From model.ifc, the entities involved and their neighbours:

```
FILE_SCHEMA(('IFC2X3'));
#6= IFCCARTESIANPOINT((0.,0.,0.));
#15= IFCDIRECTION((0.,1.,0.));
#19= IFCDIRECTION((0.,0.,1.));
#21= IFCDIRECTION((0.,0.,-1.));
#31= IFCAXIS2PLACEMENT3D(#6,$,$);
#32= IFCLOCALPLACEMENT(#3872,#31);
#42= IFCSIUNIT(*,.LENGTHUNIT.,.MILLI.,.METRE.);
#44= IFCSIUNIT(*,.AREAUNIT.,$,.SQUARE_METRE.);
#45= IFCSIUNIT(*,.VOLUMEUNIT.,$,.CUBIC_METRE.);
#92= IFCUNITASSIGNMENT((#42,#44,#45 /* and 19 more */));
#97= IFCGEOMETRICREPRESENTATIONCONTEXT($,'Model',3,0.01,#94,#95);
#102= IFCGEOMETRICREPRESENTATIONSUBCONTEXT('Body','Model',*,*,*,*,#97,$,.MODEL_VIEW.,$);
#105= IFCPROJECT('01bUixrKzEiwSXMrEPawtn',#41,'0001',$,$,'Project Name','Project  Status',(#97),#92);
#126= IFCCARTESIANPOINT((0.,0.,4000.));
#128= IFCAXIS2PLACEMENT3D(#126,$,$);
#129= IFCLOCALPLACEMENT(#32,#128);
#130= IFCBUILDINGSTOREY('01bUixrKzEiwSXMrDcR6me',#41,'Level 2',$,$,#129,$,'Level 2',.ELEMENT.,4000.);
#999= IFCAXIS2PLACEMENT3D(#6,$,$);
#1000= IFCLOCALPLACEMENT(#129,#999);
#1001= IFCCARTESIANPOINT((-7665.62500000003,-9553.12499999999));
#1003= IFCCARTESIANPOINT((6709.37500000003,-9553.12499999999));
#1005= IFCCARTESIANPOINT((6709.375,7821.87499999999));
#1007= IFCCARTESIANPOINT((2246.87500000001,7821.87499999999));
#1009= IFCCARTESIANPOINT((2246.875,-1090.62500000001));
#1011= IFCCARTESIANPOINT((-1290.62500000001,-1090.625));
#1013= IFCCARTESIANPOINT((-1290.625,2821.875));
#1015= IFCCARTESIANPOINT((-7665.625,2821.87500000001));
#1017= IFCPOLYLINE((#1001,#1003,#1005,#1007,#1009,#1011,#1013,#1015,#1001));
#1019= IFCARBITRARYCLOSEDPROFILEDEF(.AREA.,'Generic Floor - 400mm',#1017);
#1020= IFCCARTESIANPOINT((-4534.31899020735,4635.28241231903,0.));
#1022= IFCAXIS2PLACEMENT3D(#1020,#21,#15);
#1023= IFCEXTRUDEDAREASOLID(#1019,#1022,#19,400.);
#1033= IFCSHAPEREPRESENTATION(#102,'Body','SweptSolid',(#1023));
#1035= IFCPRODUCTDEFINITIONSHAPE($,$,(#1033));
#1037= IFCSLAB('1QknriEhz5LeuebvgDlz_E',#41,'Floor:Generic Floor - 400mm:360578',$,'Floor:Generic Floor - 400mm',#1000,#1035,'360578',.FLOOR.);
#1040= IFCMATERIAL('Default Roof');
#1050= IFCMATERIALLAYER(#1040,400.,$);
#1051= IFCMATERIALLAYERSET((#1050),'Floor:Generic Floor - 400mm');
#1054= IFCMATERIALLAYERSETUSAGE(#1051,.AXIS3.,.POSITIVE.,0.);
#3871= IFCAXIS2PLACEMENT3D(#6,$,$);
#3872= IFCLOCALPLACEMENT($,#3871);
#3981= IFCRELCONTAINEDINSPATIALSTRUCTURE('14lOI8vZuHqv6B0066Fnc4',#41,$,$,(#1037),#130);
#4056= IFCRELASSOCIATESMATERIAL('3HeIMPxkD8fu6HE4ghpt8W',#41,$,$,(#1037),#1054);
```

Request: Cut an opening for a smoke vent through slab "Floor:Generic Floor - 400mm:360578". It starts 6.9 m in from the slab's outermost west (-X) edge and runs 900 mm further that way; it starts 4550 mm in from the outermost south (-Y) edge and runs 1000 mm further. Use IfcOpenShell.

```python
import numpy as np
import ifcopenshell
import ifcopenshell.api.feature
import ifcopenshell.api.geometry
import ifcopenshell.api.root
import ifcopenshell.geom
import ifcopenshell.util.placement
import ifcopenshell.util.representation
import ifcopenshell.util.shape
import ifcopenshell.util.unit

model = ifcopenshell.open("model.ifc")
unit_scale = ifcopenshell.util.unit.calculate_unit_scale(model)
settings = ifcopenshell.geom.settings()


def volume(element):
    """Net volume in cubic metres, openings subtracted."""
    shape = ifcopenshell.geom.create_shape(settings, element)
    return ifcopenshell.util.shape.get_volume(shape.geometry)


slab = model.by_guid("1QknriEhz5LeuebvgDlz_E")
before = volume(slab)

# Extent in the slab's own axes, in metres. The edges named are its -X and -Y sides.
slab_shape = ifcopenshell.geom.create_shape(settings, slab)
vertices = ifcopenshell.util.shape.get_vertices(slab_shape.geometry)
x_min, y_min, bottom = vertices.min(axis=0)
top = vertices[:, 2].max()

opening = ifcopenshell.api.root.create_entity(model, ifc_class="IfcOpeningElement", name="Smoke vent opening")
context = ifcopenshell.util.representation.get_context(model, "Model", "Body", "MODEL_VIEW")
width, depth = 0.9, 1
outline = [(0.0, 0.0), (width, 0.0), (width, depth), (0.0, depth), (0.0, 0.0)]
# Overshoot both faces by 50 mm so the cut is clean.
shape = ifcopenshell.api.geometry.add_slab_representation(
    model, context=context, depth=top - bottom + 0.1, polyline=outline
)
ifcopenshell.api.geometry.assign_representation(model, product=opening, representation=shape)

matrix = ifcopenshell.util.placement.get_local_placement(slab.ObjectPlacement)
matrix[:, 3] = matrix @ np.append(np.array([x_min + 6.9, y_min + 4.55, bottom - 0.05]) / unit_scale, 1.0)
ifcopenshell.api.geometry.edit_object_placement(model, product=opening, matrix=matrix, is_si=False)
ifcopenshell.api.feature.add_feature(model, feature=opening, element=slab)

after = volume(slab)

print(f"slab volume {before:.3f} -> {after:.3f} m3")

model.write("model_rev.ifc")
```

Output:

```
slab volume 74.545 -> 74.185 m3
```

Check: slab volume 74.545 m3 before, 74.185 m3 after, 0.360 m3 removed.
